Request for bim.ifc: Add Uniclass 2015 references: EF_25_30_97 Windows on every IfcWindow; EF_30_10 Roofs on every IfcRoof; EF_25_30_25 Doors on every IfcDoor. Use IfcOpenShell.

First a look at what the model holds.

```python
import ifcopenshell

model = ifcopenshell.open("bim.ifc")
print(model.schema)
print("classifications:", [c.Name for c in model.by_type("IfcClassification")])
for ifc_class in ("IfcDoor", "IfcRoof", "IfcStair", "IfcWall", "IfcWindow"):
    print(ifc_class, len(model.by_type(ifc_class)))
```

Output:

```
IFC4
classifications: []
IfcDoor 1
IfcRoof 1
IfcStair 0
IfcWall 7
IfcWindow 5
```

```python
import ifcopenshell
import ifcopenshell.api.classification

model = ifcopenshell.open("bim.ifc")

system = ifcopenshell.api.classification.add_classification(model, classification="Uniclass 2015")

codes = {
    "IfcWindow": ("EF_25_30_97", "Windows"),
    "IfcRoof": ("EF_30_10", "Roofs"),
    "IfcDoor": ("EF_25_30_25", "Doors"),
}
for ifc_class, (code, name) in codes.items():
    products = model.by_type(ifc_class)
    ifcopenshell.api.classification.add_reference(
        model, products=products, classification=system, identification=code, name=name
    )
    print(code, len(products))

model.write("bim_updated.ifc")
```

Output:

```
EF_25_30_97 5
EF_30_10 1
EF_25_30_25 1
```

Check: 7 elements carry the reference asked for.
